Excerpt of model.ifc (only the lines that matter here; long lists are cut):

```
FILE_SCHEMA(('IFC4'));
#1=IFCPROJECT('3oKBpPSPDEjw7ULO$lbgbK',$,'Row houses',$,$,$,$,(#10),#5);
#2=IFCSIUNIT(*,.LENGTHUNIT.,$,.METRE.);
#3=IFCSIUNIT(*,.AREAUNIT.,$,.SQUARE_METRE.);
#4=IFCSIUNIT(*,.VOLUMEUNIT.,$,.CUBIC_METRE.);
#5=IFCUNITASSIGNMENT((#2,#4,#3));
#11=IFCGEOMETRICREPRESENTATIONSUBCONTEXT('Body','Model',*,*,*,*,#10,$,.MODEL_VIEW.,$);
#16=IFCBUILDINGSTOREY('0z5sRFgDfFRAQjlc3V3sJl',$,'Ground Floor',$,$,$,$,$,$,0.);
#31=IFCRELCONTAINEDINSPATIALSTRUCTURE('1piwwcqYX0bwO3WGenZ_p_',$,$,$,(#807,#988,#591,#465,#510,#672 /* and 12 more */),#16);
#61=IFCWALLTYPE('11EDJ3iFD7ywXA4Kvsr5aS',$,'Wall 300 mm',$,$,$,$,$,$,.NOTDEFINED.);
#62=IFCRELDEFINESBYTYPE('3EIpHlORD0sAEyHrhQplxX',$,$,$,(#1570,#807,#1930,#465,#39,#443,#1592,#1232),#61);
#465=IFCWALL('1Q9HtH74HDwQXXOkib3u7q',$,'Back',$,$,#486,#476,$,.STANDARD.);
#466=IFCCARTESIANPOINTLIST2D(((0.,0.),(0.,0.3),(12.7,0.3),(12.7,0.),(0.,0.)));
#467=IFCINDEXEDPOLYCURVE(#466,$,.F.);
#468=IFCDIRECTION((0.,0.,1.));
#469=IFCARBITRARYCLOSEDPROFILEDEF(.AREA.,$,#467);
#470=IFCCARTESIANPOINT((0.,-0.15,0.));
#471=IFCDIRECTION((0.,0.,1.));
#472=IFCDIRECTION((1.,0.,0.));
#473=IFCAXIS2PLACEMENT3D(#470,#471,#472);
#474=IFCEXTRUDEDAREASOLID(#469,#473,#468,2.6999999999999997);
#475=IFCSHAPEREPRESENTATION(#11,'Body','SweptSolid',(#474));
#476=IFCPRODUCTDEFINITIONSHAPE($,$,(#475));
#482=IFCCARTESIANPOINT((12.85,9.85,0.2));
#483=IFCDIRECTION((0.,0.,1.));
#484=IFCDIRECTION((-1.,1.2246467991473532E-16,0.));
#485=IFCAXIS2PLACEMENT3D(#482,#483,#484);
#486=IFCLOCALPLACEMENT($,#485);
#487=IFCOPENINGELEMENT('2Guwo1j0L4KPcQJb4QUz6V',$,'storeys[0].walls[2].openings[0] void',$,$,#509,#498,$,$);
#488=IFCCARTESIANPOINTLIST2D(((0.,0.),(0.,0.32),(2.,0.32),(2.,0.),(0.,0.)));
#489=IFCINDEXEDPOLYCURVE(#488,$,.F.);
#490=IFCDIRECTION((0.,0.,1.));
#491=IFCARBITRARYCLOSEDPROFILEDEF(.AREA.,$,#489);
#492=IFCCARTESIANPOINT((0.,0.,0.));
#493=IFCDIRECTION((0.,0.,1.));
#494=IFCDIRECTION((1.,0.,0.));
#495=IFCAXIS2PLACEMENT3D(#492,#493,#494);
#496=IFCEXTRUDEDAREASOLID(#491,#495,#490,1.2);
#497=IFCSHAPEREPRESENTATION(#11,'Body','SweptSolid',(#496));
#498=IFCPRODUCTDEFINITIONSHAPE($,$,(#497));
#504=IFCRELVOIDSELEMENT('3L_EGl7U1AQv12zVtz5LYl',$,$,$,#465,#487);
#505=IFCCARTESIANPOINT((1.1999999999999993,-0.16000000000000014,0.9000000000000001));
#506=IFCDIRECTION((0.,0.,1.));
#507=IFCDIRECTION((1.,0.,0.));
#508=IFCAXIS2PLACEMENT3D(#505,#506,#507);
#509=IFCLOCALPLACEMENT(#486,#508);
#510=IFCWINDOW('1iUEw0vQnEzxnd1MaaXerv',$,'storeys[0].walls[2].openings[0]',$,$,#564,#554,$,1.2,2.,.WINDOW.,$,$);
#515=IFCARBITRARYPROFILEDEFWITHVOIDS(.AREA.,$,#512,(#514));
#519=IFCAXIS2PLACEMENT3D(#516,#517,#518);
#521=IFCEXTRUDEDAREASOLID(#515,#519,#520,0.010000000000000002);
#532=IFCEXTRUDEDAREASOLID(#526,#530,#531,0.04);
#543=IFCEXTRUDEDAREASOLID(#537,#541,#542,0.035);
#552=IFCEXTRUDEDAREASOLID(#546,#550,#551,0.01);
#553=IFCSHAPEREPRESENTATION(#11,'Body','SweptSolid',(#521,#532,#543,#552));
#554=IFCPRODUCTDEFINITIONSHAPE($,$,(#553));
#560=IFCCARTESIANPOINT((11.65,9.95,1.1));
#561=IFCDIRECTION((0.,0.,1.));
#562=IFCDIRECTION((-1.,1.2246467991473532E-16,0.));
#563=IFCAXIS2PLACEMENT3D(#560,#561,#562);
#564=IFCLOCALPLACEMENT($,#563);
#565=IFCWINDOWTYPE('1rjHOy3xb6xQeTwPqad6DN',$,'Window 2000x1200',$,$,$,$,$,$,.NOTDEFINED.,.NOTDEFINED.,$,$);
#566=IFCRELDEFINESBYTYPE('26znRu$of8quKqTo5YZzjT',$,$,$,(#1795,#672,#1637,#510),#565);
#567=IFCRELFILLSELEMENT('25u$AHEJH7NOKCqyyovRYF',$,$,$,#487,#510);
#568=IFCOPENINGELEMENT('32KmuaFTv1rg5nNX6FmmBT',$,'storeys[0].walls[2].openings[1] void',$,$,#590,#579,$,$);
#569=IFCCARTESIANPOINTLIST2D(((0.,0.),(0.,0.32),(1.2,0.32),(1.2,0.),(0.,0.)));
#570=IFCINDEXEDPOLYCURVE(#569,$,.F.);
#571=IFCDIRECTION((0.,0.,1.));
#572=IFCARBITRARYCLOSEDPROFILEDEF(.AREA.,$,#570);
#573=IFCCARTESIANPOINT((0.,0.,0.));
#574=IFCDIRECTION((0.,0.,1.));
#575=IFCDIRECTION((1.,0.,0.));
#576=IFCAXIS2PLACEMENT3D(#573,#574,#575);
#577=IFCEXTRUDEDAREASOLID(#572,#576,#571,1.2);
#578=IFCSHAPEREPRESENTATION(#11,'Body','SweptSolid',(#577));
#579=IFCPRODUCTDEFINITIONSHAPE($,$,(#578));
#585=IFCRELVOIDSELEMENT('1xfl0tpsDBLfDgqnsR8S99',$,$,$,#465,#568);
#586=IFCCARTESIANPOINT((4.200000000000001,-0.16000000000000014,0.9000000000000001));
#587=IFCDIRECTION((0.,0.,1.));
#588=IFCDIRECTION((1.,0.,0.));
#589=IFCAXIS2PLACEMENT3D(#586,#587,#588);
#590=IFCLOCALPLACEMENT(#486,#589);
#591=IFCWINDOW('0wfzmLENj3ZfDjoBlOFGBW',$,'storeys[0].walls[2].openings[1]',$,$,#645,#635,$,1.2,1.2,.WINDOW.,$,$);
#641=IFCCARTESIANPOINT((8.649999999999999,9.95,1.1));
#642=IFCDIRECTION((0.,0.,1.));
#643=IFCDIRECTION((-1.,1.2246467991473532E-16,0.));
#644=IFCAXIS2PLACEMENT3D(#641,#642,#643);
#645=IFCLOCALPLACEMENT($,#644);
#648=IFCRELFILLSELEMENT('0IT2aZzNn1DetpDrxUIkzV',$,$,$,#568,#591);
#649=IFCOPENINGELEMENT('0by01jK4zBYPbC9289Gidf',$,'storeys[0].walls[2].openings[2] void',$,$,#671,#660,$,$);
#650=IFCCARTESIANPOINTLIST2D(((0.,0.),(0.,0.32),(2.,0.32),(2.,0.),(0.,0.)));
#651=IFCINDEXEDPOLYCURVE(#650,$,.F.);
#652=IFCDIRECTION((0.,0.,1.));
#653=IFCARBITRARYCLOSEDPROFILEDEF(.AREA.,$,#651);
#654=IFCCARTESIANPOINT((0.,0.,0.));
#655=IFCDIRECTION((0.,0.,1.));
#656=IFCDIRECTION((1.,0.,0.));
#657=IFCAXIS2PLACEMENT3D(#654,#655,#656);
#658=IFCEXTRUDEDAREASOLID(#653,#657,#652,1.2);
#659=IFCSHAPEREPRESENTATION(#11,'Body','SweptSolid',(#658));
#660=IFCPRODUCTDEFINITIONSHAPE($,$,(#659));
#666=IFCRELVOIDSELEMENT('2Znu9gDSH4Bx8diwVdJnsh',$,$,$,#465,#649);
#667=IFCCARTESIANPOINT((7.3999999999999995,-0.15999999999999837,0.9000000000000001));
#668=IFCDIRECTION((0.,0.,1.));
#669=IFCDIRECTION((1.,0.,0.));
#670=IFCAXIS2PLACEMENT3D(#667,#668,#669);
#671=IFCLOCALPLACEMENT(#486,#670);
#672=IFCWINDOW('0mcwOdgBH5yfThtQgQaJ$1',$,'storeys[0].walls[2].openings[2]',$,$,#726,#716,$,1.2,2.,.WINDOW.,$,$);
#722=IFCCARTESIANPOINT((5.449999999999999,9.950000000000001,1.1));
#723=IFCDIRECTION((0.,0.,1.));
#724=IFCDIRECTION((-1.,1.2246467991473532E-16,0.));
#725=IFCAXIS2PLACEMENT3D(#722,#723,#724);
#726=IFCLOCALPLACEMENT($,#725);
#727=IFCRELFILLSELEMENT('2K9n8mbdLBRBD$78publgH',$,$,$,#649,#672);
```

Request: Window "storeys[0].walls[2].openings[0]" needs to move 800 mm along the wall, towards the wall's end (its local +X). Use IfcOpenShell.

```python
import ifcopenshell
import ifcopenshell.api.geometry
import ifcopenshell.util.placement

model = ifcopenshell.open("model.ifc")

window = model.by_id(510)
opening = window.FillsVoids[0].RelatingOpeningElement
wall = opening.VoidsElements[0].RelatingBuildingElement

wall_matrix = ifcopenshell.util.placement.get_local_placement(wall.ObjectPlacement)
shift = wall_matrix[:3, 0] * 0.8
before = ifcopenshell.util.placement.get_local_placement(window.ObjectPlacement)[:3, 3].copy()

# The window is not placed relative to its opening, so move both.
for product in (opening, window):
    matrix = ifcopenshell.util.placement.get_local_placement(product.ObjectPlacement)
    matrix[:3, 3] += shift
    ifcopenshell.api.geometry.edit_object_placement(model, product=product, matrix=matrix, is_si=False)

after = ifcopenshell.util.placement.get_local_placement(window.ObjectPlacement)[:3, 3]
print("window moved by", (after - before).round(3) + 0.0)

model.write("model-out.ifc")
```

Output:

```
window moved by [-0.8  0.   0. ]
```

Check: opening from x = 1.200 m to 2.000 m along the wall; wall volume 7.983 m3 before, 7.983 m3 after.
